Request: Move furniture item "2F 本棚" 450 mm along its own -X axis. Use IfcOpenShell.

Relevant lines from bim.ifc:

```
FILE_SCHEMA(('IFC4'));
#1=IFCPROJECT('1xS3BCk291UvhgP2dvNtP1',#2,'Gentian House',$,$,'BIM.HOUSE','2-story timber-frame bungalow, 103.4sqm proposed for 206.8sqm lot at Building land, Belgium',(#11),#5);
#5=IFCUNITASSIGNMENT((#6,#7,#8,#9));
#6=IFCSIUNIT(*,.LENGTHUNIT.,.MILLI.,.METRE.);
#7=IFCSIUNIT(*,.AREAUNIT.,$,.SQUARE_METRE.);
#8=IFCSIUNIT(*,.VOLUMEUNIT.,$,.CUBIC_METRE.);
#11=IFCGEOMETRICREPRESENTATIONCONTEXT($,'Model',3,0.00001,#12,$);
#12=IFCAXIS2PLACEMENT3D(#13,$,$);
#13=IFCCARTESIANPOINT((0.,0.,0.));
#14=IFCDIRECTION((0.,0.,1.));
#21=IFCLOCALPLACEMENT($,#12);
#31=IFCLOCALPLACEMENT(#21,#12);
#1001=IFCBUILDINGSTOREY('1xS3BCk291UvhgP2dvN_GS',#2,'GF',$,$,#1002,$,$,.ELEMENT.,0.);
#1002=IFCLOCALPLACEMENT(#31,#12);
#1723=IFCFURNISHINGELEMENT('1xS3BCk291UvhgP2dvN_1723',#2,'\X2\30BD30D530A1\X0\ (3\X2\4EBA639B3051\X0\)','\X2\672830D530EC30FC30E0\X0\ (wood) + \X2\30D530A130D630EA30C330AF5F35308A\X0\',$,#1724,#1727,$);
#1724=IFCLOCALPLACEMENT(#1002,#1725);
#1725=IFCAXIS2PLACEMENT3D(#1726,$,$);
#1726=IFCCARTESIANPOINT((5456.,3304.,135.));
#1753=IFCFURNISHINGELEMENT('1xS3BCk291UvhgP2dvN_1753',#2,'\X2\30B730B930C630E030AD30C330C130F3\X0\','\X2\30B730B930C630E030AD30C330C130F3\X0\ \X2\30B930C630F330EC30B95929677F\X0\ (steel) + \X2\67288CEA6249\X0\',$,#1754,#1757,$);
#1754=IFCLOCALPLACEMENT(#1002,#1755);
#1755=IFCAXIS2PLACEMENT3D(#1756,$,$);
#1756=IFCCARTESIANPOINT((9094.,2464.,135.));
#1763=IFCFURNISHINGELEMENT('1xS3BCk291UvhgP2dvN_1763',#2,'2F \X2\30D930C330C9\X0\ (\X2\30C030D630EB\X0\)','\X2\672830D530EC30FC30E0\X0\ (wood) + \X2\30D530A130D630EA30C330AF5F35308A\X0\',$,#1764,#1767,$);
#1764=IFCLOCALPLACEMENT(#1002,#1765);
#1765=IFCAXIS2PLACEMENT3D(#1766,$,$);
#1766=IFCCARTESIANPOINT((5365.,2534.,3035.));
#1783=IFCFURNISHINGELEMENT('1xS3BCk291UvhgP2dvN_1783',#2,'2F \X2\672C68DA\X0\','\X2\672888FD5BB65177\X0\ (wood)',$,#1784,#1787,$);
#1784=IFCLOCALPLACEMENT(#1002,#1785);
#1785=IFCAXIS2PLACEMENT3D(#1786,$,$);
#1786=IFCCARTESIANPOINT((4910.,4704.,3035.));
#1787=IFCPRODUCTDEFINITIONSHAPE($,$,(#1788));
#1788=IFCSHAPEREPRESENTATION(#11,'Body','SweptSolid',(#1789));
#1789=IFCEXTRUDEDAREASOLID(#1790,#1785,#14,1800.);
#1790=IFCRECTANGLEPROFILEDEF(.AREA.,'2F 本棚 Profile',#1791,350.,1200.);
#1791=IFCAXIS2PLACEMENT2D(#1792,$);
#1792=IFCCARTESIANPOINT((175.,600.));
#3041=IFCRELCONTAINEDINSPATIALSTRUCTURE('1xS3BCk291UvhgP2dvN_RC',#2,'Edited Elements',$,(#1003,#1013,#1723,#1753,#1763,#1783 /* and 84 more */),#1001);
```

```python
import ifcopenshell
import ifcopenshell.api.geometry
import ifcopenshell.util.placement
import ifcopenshell.util.unit

model = ifcopenshell.open("bim.ifc")
unit_scale = ifcopenshell.util.unit.calculate_unit_scale(model)

item = model.by_guid("1xS3BCk291UvhgP2dvN_1783")
matrix = ifcopenshell.util.placement.get_local_placement(item.ObjectPlacement)
matrix[:3, 3] -= matrix[:3, 0] * 0.45 / unit_scale
ifcopenshell.api.geometry.edit_object_placement(model, product=item, matrix=matrix, is_si=False)

print(ifcopenshell.util.placement.get_local_placement(item.ObjectPlacement).round(3) + 0.0)

model.write("bim_edited.ifc")
```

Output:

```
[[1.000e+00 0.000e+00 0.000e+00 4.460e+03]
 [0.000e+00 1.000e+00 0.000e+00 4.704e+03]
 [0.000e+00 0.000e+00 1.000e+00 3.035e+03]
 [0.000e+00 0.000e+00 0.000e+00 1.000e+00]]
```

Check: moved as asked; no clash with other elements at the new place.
